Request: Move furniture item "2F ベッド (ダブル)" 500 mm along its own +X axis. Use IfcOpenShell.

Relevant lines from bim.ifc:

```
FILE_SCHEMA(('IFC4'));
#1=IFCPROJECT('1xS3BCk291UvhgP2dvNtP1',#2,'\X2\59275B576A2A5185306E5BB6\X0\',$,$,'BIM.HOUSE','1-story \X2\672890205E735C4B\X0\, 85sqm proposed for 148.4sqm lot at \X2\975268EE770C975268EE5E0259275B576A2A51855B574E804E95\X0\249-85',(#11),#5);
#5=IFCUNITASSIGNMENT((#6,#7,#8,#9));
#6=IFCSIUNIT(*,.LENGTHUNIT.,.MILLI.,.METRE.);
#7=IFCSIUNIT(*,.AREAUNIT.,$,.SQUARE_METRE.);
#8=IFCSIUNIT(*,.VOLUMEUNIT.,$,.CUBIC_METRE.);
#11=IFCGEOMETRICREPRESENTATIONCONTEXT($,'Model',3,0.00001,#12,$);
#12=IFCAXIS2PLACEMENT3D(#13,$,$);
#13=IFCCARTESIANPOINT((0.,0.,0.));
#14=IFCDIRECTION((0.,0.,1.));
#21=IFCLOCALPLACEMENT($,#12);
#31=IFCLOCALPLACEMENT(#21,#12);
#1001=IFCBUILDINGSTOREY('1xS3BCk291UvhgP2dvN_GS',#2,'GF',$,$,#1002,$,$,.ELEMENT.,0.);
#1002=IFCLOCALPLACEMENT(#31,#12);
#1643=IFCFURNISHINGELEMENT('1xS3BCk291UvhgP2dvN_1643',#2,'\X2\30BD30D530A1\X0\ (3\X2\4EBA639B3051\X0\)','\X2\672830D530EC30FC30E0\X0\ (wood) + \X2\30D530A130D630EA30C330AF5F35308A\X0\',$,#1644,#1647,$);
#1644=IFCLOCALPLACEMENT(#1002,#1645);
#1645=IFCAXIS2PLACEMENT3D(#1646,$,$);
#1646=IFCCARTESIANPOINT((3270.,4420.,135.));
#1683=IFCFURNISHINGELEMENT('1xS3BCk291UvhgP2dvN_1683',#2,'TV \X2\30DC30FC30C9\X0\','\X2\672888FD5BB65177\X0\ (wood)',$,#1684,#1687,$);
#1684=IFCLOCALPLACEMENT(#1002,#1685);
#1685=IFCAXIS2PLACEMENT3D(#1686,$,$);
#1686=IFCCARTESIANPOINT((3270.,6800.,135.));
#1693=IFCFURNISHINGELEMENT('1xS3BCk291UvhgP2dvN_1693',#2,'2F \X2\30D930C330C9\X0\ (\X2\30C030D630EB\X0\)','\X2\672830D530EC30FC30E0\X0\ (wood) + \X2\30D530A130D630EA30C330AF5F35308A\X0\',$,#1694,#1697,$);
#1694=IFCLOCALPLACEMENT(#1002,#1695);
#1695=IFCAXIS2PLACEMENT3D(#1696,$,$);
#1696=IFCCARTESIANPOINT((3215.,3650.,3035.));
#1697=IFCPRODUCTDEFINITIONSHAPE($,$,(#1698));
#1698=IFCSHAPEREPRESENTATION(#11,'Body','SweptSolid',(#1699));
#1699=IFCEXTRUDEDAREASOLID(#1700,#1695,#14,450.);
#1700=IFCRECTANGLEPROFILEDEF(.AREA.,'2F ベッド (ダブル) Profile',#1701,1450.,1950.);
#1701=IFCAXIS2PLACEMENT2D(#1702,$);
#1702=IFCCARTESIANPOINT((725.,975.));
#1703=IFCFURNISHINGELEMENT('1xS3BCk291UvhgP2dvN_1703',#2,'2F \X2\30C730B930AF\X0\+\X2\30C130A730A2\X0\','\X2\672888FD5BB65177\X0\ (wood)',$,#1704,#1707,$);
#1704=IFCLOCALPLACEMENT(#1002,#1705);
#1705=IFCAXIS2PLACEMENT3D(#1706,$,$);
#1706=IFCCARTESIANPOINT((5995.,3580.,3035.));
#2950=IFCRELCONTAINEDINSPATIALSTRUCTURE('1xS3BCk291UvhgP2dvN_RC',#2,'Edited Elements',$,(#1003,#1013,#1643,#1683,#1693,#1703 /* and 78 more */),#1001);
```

```python
import ifcopenshell
import ifcopenshell.api.geometry
import ifcopenshell.util.placement

model = ifcopenshell.open("bim.ifc")

item = model.by_id(1693)
matrix = ifcopenshell.util.placement.get_local_placement(item.ObjectPlacement)
matrix[:3, 3] += matrix[:3, 0] * 500.0
ifcopenshell.api.geometry.edit_object_placement(model, product=item, matrix=matrix, is_si=False)

print(ifcopenshell.util.placement.get_local_placement(item.ObjectPlacement).round(3) + 0.0)

model.write("bim_edited.ifc")
```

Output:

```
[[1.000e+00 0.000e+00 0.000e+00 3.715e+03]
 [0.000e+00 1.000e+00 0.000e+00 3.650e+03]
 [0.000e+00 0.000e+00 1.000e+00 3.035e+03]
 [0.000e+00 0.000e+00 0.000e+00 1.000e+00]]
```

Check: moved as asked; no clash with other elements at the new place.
